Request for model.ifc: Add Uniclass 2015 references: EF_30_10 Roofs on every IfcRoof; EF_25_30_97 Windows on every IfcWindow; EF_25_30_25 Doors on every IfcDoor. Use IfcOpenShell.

First a look at what the model holds.

```python
import ifcopenshell

model = ifcopenshell.open("model.ifc")
print(model.schema)
print("classifications:", [c.Name for c in model.by_type("IfcClassification")])
for ifc_class in ("IfcDoor", "IfcRoof", "IfcStair", "IfcWall", "IfcWindow"):
    print(ifc_class, len(model.by_type(ifc_class)))
```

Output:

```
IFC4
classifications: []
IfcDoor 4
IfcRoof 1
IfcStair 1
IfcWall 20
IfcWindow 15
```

```python
import ifcopenshell
import ifcopenshell.api.classification

model = ifcopenshell.open("model.ifc")

system = ifcopenshell.api.classification.add_classification(model, classification="Uniclass 2015")

codes = {
    "IfcRoof": ("EF_30_10", "Roofs"),
    "IfcWindow": ("EF_25_30_97", "Windows"),
    "IfcDoor": ("EF_25_30_25", "Doors"),
}
for ifc_class, (code, name) in codes.items():
    products = model.by_type(ifc_class)
    ifcopenshell.api.classification.add_reference(
        model, products=products, classification=system, identification=code, name=name
    )
    print(code, len(products))

model.write("model-out.ifc")
```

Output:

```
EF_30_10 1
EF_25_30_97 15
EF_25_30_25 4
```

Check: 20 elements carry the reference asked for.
